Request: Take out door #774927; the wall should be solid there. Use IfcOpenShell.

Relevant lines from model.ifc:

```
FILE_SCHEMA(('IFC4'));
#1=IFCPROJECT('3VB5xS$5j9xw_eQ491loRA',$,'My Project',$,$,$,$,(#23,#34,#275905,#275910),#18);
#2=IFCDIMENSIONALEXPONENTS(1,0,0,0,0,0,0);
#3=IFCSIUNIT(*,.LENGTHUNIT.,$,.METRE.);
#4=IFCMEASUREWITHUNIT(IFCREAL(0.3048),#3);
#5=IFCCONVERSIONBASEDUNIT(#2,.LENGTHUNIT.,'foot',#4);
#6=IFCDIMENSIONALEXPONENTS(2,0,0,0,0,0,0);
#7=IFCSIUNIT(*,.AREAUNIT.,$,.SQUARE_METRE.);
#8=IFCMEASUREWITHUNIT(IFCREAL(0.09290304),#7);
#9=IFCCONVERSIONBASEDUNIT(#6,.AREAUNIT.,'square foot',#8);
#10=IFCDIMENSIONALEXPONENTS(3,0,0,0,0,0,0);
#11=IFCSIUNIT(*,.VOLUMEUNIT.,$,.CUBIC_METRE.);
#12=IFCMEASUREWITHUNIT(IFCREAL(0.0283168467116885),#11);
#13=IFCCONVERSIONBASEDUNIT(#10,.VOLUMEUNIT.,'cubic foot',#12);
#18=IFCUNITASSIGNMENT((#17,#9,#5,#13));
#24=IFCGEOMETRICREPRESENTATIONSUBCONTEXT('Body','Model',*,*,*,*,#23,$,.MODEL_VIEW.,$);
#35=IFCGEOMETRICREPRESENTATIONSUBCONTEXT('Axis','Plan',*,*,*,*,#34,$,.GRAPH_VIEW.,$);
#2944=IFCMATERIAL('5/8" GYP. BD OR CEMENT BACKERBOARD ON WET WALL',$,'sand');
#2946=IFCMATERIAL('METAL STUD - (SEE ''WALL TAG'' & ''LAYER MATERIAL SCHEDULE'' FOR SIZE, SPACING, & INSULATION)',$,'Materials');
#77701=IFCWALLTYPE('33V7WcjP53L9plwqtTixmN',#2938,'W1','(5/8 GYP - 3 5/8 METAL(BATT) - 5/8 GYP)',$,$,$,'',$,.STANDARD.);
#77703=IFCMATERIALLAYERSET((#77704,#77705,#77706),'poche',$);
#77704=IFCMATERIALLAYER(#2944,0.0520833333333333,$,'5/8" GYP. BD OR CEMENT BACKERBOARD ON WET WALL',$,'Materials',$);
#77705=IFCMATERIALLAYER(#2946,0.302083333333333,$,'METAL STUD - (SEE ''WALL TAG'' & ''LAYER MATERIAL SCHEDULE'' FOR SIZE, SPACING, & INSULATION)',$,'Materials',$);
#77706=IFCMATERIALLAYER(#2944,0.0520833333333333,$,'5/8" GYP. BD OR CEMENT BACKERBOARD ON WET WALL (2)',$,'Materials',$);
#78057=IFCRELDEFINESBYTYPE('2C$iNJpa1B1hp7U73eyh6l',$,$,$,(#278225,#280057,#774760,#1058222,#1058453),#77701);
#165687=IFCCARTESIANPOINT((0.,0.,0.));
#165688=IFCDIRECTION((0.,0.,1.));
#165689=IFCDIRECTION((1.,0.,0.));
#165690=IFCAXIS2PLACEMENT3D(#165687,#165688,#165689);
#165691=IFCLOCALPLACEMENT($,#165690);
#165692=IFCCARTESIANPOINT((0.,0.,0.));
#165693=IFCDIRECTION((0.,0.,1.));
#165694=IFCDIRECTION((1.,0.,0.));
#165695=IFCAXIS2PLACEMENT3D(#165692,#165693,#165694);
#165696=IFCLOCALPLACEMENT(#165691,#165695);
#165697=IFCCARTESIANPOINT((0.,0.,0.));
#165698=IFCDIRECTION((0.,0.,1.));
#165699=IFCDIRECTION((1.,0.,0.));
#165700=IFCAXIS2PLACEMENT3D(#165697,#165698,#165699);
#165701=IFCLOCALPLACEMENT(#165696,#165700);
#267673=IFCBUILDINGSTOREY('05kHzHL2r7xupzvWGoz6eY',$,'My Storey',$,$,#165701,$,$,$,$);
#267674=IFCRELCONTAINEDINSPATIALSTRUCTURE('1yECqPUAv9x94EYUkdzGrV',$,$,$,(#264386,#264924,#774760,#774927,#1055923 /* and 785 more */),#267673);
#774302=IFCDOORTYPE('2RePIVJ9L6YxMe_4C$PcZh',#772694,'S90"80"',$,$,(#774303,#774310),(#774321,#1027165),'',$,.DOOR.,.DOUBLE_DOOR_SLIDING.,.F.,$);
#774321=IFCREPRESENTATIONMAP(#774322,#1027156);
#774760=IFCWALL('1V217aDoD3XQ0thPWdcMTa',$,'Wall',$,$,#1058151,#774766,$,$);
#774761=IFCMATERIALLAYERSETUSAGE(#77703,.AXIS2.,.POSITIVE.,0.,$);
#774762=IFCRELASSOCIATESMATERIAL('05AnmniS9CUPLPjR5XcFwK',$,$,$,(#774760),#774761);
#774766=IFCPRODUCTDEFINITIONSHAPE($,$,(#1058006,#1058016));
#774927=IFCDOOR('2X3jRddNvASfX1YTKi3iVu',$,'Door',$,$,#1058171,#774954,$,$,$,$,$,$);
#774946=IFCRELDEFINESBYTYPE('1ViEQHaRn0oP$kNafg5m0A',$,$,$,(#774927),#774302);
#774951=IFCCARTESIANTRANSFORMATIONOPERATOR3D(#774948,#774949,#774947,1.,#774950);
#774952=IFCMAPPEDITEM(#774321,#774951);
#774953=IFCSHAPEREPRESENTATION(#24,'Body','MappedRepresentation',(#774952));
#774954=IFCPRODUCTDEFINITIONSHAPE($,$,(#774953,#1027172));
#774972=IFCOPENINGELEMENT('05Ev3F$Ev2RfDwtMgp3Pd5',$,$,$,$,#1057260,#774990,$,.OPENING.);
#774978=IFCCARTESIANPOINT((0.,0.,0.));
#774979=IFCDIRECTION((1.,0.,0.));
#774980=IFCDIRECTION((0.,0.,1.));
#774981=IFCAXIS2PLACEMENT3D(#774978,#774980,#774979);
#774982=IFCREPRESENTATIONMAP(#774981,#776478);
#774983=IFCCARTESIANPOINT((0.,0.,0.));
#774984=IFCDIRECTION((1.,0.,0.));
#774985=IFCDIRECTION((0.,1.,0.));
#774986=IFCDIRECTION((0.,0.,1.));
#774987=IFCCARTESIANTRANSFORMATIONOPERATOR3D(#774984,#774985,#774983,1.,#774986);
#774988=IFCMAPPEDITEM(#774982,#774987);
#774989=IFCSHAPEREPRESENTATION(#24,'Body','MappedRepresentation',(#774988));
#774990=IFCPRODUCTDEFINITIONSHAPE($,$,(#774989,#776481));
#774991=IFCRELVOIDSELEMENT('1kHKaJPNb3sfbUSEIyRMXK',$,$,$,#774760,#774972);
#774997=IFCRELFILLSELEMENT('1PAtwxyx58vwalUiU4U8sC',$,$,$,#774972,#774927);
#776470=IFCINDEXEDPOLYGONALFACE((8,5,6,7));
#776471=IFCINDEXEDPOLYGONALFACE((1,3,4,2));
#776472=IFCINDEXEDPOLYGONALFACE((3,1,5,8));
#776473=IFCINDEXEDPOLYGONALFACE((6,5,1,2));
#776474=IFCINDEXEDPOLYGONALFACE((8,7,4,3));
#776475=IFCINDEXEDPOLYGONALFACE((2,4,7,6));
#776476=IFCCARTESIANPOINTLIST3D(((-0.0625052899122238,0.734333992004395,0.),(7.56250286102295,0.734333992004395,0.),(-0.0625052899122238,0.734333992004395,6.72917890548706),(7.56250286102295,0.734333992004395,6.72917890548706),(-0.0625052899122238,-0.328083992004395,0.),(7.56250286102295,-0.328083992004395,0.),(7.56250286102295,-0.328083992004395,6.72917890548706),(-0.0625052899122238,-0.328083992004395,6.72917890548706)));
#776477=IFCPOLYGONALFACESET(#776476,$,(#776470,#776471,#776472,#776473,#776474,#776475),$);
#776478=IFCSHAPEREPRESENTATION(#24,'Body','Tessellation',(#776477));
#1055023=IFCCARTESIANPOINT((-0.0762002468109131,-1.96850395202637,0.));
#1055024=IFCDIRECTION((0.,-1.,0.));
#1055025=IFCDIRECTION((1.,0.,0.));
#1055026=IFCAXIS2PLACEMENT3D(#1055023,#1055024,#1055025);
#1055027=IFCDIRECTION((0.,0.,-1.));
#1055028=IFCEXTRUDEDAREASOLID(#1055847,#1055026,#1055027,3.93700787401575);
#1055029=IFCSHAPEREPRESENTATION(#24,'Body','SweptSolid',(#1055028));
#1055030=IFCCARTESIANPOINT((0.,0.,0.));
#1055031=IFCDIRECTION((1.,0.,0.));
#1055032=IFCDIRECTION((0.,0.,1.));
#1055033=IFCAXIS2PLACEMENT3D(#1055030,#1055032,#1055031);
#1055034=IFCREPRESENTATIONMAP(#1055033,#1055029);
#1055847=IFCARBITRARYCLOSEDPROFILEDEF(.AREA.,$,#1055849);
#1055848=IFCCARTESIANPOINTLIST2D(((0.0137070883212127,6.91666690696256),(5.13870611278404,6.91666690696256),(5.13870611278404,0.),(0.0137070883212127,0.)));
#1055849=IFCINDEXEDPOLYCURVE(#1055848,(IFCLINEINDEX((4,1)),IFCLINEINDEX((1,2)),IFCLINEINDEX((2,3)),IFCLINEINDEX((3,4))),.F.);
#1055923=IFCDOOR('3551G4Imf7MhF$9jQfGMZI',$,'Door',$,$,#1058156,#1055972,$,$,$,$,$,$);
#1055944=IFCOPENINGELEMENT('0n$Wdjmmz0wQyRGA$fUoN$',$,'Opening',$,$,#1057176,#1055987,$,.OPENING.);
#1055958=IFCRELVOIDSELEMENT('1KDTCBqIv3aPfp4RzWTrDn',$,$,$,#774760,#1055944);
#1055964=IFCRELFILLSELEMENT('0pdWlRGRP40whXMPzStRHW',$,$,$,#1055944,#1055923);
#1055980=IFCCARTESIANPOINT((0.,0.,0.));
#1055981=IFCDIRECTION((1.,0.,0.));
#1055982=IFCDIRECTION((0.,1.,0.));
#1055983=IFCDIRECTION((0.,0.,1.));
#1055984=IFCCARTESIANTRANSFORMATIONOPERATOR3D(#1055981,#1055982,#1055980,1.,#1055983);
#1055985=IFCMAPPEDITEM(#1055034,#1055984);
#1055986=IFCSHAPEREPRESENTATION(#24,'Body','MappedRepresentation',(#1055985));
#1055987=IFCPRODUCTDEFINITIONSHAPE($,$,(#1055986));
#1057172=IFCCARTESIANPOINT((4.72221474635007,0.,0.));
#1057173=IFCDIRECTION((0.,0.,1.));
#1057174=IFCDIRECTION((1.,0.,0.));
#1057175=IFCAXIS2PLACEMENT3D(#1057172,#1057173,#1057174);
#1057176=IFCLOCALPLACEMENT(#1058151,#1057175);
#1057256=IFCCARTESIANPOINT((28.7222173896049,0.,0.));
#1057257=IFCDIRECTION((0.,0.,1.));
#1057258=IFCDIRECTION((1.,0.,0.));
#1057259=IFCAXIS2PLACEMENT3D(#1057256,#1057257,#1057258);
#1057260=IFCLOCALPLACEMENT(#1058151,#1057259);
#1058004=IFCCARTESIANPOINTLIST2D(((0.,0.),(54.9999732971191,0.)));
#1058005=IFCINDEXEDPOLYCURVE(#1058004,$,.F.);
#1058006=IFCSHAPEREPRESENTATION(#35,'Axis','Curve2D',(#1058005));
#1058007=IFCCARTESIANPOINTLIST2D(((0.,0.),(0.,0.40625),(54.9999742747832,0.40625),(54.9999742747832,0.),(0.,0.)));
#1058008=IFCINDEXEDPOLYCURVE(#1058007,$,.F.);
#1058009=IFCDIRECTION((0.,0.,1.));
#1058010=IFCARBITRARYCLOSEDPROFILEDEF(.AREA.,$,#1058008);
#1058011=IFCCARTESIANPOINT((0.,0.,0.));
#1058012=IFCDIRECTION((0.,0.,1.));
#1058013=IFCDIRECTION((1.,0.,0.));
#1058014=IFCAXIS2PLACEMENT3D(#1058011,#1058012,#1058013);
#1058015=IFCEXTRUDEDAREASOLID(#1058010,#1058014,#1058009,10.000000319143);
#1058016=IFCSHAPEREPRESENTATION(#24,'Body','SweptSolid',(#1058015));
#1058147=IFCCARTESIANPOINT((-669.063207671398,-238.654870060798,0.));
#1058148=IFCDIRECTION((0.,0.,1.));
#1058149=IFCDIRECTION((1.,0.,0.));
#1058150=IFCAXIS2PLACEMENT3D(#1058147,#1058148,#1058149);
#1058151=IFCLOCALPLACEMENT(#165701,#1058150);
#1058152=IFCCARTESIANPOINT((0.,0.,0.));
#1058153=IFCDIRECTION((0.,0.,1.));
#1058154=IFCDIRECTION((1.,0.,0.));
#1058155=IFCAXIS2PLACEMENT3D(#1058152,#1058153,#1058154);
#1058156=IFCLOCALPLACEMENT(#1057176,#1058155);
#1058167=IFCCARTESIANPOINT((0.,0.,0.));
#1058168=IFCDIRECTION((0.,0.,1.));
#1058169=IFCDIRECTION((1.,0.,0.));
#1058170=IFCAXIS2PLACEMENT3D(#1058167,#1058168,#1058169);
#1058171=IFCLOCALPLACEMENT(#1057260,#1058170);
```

```python
import ifcopenshell
import ifcopenshell.api.feature
import ifcopenshell.api.root
import ifcopenshell.geom
import ifcopenshell.util.shape

model = ifcopenshell.open("model.ifc")
settings = ifcopenshell.geom.settings()


def volume(element):
    """Net volume in cubic metres, openings subtracted."""
    shape = ifcopenshell.geom.create_shape(settings, element)
    return ifcopenshell.util.shape.get_volume(shape.geometry)


door = model.by_id(774927)
opening = door.FillsVoids[0].RelatingOpeningElement
wall = opening.VoidsElements[0].RelatingBuildingElement
before = volume(wall)

ifcopenshell.api.root.remove_product(model, product=door)
ifcopenshell.api.feature.remove_feature(model, feature=opening)

after = volume(wall)

print(f"wall volume {before:.3f} -> {after:.3f} m3")

model.write("model_rev.ifc")
```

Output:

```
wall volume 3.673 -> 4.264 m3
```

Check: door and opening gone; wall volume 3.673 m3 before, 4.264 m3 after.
